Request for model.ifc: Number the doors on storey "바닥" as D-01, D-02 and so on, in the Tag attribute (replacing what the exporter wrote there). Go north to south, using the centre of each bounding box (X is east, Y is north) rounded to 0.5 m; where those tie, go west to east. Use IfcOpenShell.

First a look at what the model holds.

```python
import ifcopenshell
import ifcopenshell.util.element
import ifcopenshell.util.placement

model = ifcopenshell.open("model.ifc")
print(model.schema)
storey = next(s for s in model.by_type("IfcBuildingStorey") if s.Name == "바닥")
doors = [e for e in ifcopenshell.util.element.get_decomposition(storey) if e.is_a("IfcDoor")]
for e in sorted(doors, key=lambda e: e.id()):
    origin = ifcopenshell.util.placement.get_local_placement(e.ObjectPlacement)[:3, 3]
    print(e.id(), e.Tag, e.Name, origin.round(2) + 0.0, sep=" | ")
```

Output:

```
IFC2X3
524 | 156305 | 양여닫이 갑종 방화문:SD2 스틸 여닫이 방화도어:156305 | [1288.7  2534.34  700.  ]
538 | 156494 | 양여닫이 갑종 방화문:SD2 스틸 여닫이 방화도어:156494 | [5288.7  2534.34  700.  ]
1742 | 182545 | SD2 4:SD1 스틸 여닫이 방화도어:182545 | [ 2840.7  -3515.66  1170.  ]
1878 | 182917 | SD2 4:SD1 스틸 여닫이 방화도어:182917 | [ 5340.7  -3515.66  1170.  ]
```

```python
import ifcopenshell
import ifcopenshell.geom
import ifcopenshell.util.element
import ifcopenshell.util.shape

model = ifcopenshell.open("model.ifc")
settings = ifcopenshell.geom.settings()
settings.set("use-world-coords", True)


def centre(element):
    shape = ifcopenshell.geom.create_shape(settings, element)
    return ifcopenshell.util.shape.get_bbox_centroid(shape.geometry)


storey = next(s for s in model.by_type("IfcBuildingStorey") if s.Name == "바닥")
doors = [e for e in ifcopenshell.util.element.get_decomposition(storey) if e.is_a("IfcDoor")]

# Insertion points can sit at a corner or the storey origin, so sort by the geometry (in metres).
centres = {e: centre(e) for e in doors}
doors.sort(key=lambda e: (-round(centres[e][1] / 0.5), centres[e][0]))

for i, e in enumerate(doors, start=1):
    number = f"D-{i:02d}"
    e.Tag = number
    print(e.id(), number)

model.write("model_v2.ifc")
```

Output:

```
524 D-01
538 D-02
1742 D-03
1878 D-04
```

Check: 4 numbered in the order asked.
